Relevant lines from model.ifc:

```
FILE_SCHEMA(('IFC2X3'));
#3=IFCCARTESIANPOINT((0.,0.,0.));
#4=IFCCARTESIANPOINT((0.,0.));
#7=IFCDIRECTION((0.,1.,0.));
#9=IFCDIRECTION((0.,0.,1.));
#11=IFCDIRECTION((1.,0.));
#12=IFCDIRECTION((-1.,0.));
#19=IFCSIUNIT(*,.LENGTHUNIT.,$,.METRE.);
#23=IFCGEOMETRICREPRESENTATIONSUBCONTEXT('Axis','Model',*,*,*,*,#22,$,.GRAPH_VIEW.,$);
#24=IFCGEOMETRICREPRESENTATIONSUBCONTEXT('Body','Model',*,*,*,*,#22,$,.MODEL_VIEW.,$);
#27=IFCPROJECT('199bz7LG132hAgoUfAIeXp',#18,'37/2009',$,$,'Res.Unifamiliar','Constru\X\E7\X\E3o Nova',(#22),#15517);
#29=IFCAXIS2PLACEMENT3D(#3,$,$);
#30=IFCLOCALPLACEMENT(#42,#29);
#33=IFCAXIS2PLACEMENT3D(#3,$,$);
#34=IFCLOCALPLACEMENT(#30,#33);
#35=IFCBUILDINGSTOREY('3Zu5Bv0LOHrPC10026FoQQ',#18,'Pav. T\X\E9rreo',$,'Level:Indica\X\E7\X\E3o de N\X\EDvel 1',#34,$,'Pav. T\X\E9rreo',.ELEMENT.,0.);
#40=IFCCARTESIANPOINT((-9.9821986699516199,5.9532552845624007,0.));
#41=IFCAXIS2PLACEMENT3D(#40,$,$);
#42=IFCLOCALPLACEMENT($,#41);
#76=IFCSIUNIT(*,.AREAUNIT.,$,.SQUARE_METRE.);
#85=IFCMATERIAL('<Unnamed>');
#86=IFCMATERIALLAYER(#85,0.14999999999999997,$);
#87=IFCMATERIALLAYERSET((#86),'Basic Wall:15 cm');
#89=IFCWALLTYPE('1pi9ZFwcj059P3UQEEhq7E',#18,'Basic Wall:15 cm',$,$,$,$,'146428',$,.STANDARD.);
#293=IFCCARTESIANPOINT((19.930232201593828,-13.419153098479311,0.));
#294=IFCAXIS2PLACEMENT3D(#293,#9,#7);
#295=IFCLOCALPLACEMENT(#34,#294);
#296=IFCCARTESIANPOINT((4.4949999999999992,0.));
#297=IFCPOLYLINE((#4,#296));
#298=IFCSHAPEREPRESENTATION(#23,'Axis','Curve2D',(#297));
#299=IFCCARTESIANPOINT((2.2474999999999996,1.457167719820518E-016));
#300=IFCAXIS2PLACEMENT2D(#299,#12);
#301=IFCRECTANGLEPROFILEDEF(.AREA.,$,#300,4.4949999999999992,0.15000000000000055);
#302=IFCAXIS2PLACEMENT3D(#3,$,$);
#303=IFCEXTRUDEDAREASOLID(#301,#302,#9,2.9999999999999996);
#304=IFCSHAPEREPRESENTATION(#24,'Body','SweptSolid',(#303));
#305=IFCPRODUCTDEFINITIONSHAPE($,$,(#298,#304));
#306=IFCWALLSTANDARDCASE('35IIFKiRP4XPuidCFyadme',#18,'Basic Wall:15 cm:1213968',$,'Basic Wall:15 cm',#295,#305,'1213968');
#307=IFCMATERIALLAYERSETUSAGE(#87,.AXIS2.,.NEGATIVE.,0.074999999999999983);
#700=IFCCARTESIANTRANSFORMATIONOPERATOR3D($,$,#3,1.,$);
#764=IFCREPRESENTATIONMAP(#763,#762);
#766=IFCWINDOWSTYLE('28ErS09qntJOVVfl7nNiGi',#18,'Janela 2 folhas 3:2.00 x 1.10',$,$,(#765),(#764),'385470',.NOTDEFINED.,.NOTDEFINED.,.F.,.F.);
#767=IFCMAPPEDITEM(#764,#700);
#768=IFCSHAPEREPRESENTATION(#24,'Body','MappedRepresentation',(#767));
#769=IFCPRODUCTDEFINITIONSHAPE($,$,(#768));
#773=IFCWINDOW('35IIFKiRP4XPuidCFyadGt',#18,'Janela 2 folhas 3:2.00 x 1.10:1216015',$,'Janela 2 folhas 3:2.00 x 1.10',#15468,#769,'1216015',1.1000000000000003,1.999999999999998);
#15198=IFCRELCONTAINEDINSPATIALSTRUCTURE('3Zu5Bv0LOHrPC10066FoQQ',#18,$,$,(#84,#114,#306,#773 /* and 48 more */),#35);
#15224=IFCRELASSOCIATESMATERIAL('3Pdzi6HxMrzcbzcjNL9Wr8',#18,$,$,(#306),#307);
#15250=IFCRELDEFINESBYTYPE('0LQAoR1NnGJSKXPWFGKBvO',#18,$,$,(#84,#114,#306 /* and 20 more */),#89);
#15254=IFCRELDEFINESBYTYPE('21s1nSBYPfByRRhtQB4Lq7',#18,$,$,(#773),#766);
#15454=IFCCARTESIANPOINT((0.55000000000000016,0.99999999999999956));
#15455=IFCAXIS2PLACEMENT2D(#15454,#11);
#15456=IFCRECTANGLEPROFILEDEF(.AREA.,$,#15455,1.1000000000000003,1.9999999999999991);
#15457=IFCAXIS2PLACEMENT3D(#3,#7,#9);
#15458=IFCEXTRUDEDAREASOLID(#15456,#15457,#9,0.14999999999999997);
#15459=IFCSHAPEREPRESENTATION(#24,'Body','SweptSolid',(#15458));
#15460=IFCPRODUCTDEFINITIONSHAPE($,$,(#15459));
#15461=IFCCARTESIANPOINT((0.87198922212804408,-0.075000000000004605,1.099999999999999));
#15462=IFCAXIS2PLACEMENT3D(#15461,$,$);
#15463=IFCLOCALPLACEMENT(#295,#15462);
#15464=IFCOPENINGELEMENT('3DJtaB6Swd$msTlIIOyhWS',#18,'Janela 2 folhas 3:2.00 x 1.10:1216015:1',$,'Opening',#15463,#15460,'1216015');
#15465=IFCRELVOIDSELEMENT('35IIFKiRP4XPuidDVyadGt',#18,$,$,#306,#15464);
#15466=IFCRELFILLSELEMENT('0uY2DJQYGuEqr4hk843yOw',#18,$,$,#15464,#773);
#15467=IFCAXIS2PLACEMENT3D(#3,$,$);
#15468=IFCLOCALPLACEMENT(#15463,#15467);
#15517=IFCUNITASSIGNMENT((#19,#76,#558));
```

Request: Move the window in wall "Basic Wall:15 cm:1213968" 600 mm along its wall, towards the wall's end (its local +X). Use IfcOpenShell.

```python
import ifcopenshell
import ifcopenshell.api.geometry
import ifcopenshell.util.placement

model = ifcopenshell.open("model.ifc")

window = model.by_guid("35IIFKiRP4XPuidCFyadGt")
opening = window.FillsVoids[0].RelatingOpeningElement
wall = opening.VoidsElements[0].RelatingBuildingElement

wall_matrix = ifcopenshell.util.placement.get_local_placement(wall.ObjectPlacement)
shift = wall_matrix[:3, 0] * 0.6
before = ifcopenshell.util.placement.get_local_placement(window.ObjectPlacement)[:3, 3].copy()

# The window is placed relative to its opening, so it follows when the opening moves.
matrix = ifcopenshell.util.placement.get_local_placement(opening.ObjectPlacement)
matrix[:3, 3] += shift
ifcopenshell.api.geometry.edit_object_placement(
    model, product=opening, matrix=matrix, is_si=False, should_transform_children=True
)

after = ifcopenshell.util.placement.get_local_placement(window.ObjectPlacement)[:3, 3]
print("window moved by", (after - before).round(3) + 0.0)

model.write("model_edited.ifc")
```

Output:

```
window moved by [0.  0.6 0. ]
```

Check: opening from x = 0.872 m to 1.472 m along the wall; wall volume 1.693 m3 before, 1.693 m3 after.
